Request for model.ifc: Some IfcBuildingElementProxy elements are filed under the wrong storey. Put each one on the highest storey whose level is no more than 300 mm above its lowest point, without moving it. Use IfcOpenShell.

First a look at what the model holds.

```python
import ifcopenshell
import ifcopenshell.util.element
import ifcopenshell.util.placement

model = ifcopenshell.open("model.ifc")
print(model.schema)
for storey in model.by_type("IfcBuildingStorey"):
    level = ifcopenshell.util.placement.get_storey_elevation(storey)
    count = sum(e.is_a("IfcBuildingElementProxy") for e in ifcopenshell.util.element.get_contained(storey))
    print(storey.id(), storey.Name, round(level, 3), count, sep=" | ")
```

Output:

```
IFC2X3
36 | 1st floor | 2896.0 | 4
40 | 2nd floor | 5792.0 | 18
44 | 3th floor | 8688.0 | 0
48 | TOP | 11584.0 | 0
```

```python
import ifcopenshell
import ifcopenshell.api.spatial
import ifcopenshell.geom
import ifcopenshell.util.element
import ifcopenshell.util.placement
import ifcopenshell.util.shape
import ifcopenshell.util.unit

model = ifcopenshell.open("model.ifc")
unit_scale = ifcopenshell.util.unit.calculate_unit_scale(model)
settings = ifcopenshell.geom.settings()

levels = sorted(
    ((ifcopenshell.util.placement.get_storey_elevation(s) * unit_scale, s) for s in model.by_type("IfcBuildingStorey")),
    key=lambda pair: pair[0],
)

for e in model.by_type("IfcBuildingElementProxy"):
    current = e.ContainedInStructure[0].RelatingStructure if e.ContainedInStructure else None
    if current is None or not current.is_a("IfcBuildingStorey"):
        continue
    shape = ifcopenshell.geom.create_shape(settings, e)
    bottom = ifcopenshell.util.shape.get_shape_bottom_elevation(shape, shape.geometry)
    below = [s for level, s in levels if level <= bottom + 0.3]
    storey = below[-1] if below else levels[0][1]
    if storey != current:
        # assign_container keeps the world position.
        ifcopenshell.api.spatial.assign_container(model, products=[e], relating_structure=storey)
        print(e.id(), current.Name, "->", storey.Name)

model.write("model-out.ifc")
```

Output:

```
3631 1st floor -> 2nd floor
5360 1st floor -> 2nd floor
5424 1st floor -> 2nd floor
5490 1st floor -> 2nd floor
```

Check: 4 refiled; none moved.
